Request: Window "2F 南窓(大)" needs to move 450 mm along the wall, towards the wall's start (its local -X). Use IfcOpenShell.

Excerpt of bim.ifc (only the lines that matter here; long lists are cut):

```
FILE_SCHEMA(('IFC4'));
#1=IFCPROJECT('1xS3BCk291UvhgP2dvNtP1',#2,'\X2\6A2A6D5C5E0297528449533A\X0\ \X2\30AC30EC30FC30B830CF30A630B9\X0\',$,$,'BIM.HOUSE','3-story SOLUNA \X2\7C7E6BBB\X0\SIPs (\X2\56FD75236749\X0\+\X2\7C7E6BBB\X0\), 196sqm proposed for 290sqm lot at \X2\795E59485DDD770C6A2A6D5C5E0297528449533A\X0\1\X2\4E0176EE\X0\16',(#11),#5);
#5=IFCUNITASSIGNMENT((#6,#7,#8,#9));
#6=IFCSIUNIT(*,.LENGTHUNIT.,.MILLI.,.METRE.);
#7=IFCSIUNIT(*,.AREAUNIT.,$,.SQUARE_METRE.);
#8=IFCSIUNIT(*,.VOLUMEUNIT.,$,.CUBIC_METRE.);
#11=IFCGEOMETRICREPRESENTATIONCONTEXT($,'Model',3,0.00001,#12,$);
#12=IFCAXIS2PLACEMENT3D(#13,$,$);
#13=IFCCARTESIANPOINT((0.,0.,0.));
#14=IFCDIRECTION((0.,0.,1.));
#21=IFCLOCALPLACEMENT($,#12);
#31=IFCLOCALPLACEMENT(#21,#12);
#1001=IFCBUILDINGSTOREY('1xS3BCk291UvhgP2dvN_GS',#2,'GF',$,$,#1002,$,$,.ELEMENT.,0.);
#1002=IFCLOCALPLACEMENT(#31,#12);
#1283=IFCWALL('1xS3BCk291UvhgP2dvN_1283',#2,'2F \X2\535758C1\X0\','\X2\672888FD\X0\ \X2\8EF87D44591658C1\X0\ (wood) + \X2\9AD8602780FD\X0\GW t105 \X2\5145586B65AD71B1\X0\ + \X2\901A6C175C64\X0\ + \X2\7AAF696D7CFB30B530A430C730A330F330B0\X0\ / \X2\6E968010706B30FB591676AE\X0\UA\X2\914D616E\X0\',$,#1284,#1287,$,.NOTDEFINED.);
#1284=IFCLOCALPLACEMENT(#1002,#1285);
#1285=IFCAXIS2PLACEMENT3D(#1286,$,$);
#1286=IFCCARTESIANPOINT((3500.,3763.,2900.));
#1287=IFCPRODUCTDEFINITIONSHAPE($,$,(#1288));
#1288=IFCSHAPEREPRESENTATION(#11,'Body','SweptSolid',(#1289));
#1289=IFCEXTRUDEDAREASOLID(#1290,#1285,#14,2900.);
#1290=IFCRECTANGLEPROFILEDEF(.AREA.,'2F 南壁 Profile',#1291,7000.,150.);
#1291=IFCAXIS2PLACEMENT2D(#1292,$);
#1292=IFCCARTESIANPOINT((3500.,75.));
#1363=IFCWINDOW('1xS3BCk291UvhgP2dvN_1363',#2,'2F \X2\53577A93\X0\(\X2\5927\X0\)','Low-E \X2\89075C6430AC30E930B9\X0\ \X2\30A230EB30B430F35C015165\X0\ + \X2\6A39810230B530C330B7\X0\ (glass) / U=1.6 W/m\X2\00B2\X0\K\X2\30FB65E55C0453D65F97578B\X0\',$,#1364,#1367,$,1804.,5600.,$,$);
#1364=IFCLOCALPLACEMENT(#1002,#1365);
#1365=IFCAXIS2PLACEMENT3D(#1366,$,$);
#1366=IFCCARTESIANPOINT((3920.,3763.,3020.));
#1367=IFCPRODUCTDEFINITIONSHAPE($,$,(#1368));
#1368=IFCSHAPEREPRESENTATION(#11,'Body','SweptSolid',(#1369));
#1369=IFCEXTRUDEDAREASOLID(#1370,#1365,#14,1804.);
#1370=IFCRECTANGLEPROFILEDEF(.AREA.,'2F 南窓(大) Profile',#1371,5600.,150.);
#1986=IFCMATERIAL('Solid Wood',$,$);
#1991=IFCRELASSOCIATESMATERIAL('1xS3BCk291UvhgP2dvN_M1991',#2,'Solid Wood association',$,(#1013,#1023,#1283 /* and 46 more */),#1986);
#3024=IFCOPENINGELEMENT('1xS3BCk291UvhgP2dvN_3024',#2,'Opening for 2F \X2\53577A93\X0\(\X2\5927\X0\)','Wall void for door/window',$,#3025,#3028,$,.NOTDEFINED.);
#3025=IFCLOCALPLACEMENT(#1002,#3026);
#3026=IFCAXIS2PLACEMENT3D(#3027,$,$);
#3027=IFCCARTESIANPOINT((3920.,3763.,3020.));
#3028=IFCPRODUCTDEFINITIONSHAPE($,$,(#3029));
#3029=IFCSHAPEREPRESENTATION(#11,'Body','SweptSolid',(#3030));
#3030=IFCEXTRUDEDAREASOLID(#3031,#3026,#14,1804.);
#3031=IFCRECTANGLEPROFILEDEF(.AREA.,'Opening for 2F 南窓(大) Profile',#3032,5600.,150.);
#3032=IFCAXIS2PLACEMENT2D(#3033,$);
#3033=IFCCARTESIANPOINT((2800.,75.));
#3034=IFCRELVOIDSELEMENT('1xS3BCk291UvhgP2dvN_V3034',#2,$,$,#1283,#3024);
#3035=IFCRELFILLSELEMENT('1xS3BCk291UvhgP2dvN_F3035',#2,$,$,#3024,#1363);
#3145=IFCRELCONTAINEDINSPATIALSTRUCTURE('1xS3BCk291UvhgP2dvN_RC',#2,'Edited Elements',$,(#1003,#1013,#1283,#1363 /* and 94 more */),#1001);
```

```python
import ifcopenshell
import ifcopenshell.api.geometry
import ifcopenshell.util.placement
import ifcopenshell.util.unit

model = ifcopenshell.open("bim.ifc")
unit_scale = ifcopenshell.util.unit.calculate_unit_scale(model)

window = model.by_guid("1xS3BCk291UvhgP2dvN_1363")
opening = window.FillsVoids[0].RelatingOpeningElement
wall = opening.VoidsElements[0].RelatingBuildingElement

wall_matrix = ifcopenshell.util.placement.get_local_placement(wall.ObjectPlacement)
shift = wall_matrix[:3, 0] * -0.45 / unit_scale
before = ifcopenshell.util.placement.get_local_placement(window.ObjectPlacement)[:3, 3].copy()

# The window is not placed relative to its opening, so move both.
for product in (opening, window):
    matrix = ifcopenshell.util.placement.get_local_placement(product.ObjectPlacement)
    matrix[:3, 3] += shift
    ifcopenshell.api.geometry.edit_object_placement(model, product=product, matrix=matrix, is_si=False)

after = ifcopenshell.util.placement.get_local_placement(window.ObjectPlacement)[:3, 3]
print("window moved by", (after - before).round(3) + 0.0)

model.write("bim_edited.ifc")
```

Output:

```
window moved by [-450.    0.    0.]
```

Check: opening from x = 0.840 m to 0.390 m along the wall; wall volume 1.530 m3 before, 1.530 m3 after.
